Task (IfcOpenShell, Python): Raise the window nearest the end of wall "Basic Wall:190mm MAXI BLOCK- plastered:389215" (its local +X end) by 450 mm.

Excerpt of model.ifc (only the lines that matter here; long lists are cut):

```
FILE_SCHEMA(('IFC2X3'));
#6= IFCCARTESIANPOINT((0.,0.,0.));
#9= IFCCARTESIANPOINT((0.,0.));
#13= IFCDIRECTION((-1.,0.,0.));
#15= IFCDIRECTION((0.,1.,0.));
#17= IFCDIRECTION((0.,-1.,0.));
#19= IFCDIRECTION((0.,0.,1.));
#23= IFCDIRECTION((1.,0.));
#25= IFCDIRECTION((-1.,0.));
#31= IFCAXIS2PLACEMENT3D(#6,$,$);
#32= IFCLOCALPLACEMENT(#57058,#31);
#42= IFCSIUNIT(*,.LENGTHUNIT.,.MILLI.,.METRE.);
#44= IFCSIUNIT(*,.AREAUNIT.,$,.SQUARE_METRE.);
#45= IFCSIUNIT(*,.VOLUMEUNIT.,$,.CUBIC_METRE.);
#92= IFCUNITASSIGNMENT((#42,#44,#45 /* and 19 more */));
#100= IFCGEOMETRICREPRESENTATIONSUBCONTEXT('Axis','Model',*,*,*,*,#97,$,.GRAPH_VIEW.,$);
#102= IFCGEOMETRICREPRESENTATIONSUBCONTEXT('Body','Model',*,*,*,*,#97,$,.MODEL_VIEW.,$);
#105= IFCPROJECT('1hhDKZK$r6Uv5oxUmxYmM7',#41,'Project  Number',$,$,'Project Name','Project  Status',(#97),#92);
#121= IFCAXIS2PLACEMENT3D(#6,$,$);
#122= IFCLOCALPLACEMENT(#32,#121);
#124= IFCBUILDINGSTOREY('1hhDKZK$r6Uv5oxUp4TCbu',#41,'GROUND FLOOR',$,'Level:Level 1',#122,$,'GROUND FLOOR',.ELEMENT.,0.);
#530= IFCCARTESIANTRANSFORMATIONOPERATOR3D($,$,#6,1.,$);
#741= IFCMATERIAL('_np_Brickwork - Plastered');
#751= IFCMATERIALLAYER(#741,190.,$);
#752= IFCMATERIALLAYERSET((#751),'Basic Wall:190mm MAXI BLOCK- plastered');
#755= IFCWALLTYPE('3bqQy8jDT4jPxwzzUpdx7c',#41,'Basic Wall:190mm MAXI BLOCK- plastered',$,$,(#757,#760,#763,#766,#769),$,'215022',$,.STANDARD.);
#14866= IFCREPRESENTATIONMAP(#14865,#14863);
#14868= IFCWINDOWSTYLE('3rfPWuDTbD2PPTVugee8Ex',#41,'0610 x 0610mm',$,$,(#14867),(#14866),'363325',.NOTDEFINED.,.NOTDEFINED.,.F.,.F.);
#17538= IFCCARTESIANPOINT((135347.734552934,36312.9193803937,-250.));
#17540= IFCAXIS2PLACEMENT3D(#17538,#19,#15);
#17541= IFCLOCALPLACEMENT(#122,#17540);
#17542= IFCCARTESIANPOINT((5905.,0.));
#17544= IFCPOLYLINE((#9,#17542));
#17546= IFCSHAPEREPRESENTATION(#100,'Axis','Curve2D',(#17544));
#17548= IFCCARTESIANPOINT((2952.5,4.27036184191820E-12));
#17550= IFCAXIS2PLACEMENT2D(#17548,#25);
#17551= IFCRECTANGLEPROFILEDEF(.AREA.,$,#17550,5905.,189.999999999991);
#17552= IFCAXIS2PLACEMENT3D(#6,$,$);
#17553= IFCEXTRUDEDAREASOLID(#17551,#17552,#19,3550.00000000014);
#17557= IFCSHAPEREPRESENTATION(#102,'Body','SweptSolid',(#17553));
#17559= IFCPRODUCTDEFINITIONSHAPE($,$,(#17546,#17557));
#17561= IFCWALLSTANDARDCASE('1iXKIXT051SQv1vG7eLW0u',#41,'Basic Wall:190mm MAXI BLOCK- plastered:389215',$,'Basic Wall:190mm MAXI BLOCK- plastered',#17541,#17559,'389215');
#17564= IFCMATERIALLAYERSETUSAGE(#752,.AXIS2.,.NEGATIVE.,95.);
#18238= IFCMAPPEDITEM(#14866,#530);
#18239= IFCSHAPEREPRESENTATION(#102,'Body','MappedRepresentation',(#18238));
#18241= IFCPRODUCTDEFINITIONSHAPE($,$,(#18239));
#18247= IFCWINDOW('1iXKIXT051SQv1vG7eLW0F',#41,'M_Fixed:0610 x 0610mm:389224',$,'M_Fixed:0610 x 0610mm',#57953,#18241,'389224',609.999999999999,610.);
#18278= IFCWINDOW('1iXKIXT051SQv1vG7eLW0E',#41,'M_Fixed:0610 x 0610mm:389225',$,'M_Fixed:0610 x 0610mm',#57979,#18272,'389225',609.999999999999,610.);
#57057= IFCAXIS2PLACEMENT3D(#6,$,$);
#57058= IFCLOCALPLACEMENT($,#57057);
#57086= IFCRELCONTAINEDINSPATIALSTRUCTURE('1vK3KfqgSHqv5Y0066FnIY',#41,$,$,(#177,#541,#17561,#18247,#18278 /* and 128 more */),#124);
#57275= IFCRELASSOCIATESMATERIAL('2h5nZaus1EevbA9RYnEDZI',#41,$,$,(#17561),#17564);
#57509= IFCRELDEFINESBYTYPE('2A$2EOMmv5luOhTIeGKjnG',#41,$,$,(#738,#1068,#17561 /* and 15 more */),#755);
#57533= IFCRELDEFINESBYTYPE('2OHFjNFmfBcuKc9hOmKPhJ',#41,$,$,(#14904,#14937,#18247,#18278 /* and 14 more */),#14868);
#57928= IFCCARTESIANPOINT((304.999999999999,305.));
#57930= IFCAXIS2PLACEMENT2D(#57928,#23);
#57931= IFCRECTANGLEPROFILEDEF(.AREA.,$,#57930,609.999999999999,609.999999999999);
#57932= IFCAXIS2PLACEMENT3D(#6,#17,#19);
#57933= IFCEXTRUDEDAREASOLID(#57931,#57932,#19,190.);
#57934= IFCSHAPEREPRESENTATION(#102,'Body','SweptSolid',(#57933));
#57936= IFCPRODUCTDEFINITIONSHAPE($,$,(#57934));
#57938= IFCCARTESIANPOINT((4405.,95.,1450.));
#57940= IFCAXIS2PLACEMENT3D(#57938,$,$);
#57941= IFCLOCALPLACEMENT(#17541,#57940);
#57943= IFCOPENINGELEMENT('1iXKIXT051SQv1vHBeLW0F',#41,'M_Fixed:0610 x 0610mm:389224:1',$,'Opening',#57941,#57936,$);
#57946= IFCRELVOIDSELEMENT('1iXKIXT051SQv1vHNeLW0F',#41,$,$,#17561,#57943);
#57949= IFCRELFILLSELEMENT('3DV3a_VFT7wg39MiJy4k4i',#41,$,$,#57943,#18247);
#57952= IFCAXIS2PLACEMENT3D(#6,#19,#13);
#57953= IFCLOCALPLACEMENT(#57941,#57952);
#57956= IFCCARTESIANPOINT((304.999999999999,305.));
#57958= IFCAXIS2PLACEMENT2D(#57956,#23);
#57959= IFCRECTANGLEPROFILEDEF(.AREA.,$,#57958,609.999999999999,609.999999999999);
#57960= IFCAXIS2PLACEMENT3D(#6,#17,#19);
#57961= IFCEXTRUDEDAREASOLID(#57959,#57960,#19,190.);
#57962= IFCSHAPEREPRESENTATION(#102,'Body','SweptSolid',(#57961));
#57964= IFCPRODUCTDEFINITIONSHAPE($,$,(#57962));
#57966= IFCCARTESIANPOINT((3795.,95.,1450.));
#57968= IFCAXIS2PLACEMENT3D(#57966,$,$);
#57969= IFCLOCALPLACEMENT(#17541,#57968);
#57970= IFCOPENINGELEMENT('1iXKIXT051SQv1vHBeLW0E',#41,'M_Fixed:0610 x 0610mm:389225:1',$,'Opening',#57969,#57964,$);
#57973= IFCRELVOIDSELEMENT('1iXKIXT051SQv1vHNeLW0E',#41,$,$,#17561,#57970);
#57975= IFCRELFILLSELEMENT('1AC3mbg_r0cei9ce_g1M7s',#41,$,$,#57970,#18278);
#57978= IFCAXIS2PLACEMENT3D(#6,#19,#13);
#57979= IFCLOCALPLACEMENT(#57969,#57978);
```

```python
import numpy as np
import ifcopenshell
import ifcopenshell.api.geometry
import ifcopenshell.util.placement
import ifcopenshell.util.unit

model = ifcopenshell.open("model.ifc")
unit_scale = ifcopenshell.util.unit.calculate_unit_scale(model)

window = model.by_guid("1iXKIXT051SQv1vG7eLW0F")
opening = window.FillsVoids[0].RelatingOpeningElement
dz = 450.0

shift = np.array([0.0, 0.0, dz])
# The window is placed relative to its opening, so it follows when the opening moves.
matrix = ifcopenshell.util.placement.get_local_placement(opening.ObjectPlacement)
matrix[:3, 3] += shift
ifcopenshell.api.geometry.edit_object_placement(
    model, product=opening, matrix=matrix, is_si=False, should_transform_children=True
)

print(f"moved by {dz * unit_scale:+.3f} m")

model.write("model_v2.ifc")
```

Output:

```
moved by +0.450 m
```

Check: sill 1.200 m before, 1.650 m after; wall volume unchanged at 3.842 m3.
